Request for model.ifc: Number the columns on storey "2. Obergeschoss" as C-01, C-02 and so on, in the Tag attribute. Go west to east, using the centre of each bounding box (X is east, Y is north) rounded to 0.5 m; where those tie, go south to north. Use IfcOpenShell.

First a look at what the model holds.

```python
import ifcopenshell
import ifcopenshell.util.element
import ifcopenshell.util.placement

model = ifcopenshell.open("model.ifc")
print(model.schema)
storey = next(s for s in model.by_type("IfcBuildingStorey") if s.Name == "2. Obergeschoss")
columns = [e for e in ifcopenshell.util.element.get_decomposition(storey) if e.is_a("IfcColumn")]
for e in sorted(columns, key=lambda e: e.id()):
    origin = ifcopenshell.util.placement.get_local_placement(e.ObjectPlacement)[:3, 3]
    print(e.id(), e.Tag, e.Name, origin.round(2) + 0.0, sep=" | ")
```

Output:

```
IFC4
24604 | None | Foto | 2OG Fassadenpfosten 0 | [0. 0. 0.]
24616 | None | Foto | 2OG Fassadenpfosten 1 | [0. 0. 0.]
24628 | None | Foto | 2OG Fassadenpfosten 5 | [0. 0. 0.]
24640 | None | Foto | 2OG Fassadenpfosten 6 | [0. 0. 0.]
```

```python
import ifcopenshell
import ifcopenshell.geom
import ifcopenshell.util.element
import ifcopenshell.util.shape

model = ifcopenshell.open("model.ifc")
settings = ifcopenshell.geom.settings()
settings.set("use-world-coords", True)


def centre(element):
    shape = ifcopenshell.geom.create_shape(settings, element)
    return ifcopenshell.util.shape.get_bbox_centroid(shape.geometry)


storey = next(s for s in model.by_type("IfcBuildingStorey") if s.Name == "2. Obergeschoss")
columns = [e for e in ifcopenshell.util.element.get_decomposition(storey) if e.is_a("IfcColumn")]

# Insertion points can sit at a corner or the storey origin, so sort by the geometry (in metres).
centres = {e: centre(e) for e in columns}
columns.sort(key=lambda e: (round(centres[e][0] / 0.5), centres[e][1]))

for i, e in enumerate(columns, start=1):
    number = f"C-{i:02d}"
    e.Tag = number
    print(e.id(), number)

model.write("model_edited.ifc")
```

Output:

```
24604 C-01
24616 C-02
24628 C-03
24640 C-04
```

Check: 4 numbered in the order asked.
